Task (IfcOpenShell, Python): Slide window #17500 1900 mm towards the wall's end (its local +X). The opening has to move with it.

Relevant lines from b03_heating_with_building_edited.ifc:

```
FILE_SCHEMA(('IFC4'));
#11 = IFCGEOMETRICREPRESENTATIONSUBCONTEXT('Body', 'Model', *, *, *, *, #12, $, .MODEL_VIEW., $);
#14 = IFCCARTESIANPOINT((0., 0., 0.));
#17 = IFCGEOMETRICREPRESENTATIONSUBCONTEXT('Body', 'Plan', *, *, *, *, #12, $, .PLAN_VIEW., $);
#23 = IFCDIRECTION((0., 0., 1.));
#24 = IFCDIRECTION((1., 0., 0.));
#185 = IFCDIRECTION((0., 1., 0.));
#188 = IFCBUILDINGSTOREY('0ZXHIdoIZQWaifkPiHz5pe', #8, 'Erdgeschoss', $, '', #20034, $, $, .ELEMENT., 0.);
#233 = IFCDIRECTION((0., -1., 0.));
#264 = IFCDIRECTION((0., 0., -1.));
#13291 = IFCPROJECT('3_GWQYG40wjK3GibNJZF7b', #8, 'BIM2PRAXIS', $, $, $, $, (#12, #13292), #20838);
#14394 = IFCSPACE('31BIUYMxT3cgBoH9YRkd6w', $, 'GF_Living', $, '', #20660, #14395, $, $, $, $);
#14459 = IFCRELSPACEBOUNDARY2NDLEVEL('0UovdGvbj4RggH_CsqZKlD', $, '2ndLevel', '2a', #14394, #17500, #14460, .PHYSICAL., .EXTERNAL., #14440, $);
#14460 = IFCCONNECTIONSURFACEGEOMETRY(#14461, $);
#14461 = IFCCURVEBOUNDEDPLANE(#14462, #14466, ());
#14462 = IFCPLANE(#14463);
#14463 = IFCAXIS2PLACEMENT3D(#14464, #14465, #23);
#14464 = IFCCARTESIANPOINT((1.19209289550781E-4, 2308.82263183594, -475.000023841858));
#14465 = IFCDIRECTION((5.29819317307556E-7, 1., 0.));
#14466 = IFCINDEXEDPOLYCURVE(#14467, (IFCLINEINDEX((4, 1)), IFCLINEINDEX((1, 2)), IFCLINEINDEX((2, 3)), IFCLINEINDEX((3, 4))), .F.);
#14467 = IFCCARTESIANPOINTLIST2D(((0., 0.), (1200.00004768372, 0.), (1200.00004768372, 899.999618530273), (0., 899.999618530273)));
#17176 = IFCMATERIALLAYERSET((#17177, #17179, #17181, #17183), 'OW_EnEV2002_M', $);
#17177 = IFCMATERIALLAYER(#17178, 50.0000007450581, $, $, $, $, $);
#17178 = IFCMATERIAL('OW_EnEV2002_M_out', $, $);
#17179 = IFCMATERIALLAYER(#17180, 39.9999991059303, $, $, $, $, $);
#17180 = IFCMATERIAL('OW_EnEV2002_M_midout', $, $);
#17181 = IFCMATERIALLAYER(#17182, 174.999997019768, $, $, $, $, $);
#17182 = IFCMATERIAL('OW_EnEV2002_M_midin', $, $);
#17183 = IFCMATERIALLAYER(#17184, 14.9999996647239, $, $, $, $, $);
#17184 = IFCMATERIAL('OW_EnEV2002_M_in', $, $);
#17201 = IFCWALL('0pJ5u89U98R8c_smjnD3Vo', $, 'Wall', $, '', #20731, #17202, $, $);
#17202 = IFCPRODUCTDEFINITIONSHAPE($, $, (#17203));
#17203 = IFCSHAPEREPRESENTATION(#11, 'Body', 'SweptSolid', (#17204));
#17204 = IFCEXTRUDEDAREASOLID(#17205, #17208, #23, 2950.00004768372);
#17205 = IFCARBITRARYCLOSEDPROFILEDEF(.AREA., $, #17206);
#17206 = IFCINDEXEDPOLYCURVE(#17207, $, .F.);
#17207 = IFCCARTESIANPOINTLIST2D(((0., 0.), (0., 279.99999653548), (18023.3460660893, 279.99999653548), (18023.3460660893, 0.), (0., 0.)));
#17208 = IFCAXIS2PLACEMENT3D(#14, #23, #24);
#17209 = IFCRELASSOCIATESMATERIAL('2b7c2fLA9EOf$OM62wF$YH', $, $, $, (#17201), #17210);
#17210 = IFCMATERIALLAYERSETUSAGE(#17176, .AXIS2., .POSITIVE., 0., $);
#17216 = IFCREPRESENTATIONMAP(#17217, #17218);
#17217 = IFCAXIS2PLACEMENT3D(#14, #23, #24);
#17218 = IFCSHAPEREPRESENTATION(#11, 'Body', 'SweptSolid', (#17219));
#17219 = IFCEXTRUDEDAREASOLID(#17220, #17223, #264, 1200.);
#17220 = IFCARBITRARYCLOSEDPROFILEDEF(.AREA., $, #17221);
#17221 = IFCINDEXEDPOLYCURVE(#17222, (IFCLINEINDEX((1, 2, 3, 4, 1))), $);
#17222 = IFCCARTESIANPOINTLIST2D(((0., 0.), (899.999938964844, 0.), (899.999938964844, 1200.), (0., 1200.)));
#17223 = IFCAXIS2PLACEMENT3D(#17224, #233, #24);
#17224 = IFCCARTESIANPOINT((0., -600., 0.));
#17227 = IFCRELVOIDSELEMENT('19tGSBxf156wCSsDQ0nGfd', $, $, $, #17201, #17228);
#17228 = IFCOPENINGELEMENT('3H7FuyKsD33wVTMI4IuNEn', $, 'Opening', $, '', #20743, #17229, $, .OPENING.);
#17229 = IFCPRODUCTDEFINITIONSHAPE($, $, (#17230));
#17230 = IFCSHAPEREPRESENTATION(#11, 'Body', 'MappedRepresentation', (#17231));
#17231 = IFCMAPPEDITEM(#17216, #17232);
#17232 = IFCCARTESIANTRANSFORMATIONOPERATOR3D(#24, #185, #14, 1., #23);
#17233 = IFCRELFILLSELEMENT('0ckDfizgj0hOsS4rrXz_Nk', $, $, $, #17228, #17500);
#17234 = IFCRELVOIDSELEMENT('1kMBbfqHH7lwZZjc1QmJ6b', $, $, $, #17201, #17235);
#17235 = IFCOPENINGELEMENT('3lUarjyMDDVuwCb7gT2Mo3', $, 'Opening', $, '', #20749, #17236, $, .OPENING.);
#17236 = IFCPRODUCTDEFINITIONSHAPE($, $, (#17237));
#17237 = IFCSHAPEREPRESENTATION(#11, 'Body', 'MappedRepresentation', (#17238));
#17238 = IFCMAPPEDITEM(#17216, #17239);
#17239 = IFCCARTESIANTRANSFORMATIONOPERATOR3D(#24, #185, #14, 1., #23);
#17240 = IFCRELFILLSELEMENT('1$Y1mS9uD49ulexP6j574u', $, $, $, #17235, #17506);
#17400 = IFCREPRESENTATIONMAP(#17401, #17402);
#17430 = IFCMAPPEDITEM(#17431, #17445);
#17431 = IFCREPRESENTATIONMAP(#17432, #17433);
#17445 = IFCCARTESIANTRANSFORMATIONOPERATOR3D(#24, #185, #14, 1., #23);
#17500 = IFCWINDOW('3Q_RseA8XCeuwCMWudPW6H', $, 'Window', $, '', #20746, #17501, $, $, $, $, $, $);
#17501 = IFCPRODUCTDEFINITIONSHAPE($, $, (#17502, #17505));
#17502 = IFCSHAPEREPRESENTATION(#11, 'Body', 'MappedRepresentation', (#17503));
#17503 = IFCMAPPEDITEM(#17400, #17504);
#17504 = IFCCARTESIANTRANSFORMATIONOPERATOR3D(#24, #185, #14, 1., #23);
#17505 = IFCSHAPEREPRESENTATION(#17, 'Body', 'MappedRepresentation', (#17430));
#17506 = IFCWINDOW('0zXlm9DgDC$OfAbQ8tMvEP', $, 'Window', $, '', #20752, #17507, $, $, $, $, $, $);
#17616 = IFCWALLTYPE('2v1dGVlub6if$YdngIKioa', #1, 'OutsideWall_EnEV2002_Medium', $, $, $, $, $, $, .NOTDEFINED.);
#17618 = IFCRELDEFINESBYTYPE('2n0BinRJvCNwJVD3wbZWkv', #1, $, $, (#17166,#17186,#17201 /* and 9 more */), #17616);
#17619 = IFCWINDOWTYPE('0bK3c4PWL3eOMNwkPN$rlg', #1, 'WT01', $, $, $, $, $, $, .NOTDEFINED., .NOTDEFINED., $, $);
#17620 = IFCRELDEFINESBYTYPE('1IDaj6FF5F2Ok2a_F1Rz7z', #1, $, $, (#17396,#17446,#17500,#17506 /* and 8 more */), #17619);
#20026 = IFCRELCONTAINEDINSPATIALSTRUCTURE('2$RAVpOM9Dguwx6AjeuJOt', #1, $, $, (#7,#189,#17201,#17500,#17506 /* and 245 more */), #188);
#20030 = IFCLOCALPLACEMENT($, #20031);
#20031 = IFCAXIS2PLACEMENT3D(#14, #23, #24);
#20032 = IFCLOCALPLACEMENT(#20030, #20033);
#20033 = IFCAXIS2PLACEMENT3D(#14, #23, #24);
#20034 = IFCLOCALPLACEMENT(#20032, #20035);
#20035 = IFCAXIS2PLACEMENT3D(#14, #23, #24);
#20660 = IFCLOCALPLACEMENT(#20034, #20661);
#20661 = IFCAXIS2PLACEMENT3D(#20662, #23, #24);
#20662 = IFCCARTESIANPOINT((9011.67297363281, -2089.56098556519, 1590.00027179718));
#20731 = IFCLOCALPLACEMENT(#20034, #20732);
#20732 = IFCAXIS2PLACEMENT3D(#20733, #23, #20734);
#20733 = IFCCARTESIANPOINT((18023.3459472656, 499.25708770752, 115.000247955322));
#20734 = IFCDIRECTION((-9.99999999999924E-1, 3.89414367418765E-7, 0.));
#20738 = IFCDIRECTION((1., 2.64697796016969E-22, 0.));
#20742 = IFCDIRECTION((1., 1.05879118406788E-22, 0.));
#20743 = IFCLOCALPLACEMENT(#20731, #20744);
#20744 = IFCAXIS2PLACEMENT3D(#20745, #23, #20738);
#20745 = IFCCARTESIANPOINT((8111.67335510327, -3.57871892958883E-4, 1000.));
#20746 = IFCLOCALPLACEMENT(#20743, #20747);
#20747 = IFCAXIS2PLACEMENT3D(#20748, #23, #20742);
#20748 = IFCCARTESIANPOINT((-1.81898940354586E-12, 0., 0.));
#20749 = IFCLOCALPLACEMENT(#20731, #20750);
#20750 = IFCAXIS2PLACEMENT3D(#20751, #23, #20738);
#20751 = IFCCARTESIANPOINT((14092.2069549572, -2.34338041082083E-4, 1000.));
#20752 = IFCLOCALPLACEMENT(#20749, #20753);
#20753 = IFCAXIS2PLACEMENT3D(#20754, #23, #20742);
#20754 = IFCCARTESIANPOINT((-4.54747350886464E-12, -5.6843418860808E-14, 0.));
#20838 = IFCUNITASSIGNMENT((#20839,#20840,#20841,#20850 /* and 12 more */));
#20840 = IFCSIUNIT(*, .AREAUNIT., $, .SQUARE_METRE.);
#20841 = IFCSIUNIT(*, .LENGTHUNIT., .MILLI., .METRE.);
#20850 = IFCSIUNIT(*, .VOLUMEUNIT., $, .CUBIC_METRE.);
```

```python
import numpy as np
import ifcopenshell
import ifcopenshell.api.geometry
import ifcopenshell.util.placement
import ifcopenshell.util.unit

model = ifcopenshell.open("b03_heating_with_building_edited.ifc")
unit_scale = ifcopenshell.util.unit.calculate_unit_scale(model)

window = model.by_id(17500)
opening = window.FillsVoids[0].RelatingOpeningElement
wall = opening.VoidsElements[0].RelatingBuildingElement

wall_matrix = ifcopenshell.util.placement.get_local_placement(wall.ObjectPlacement)
shift = wall_matrix[:3, 0] * 1.9 / unit_scale
before = ifcopenshell.util.placement.get_local_placement(window.ObjectPlacement)[:3, 3].copy()

# The window is placed relative to its opening, so it follows when the opening moves.
matrix = ifcopenshell.util.placement.get_local_placement(opening.ObjectPlacement)
matrix[:3, 3] += shift
ifcopenshell.api.geometry.edit_object_placement(
    model, product=opening, matrix=matrix, is_si=False, should_transform_children=True
)

# Space boundary surfaces are stored in each space's coordinates; move them too.
for rel in window.ProvidesBoundaries:
    if not rel.ConnectionGeometry:
        continue
    surface = rel.ConnectionGeometry.SurfaceOnRelatingElement.BasisSurface
    space_matrix = ifcopenshell.util.placement.get_local_placement(rel.RelatingSpace.ObjectPlacement)
    point = np.array(surface.Position.Location.Coordinates) + space_matrix[:3, :3].T @ shift
    surface.Position = model.createIfcAxis2Placement3D(
        model.createIfcCartesianPoint(point.tolist()), surface.Position.Axis, surface.Position.RefDirection
    )

after = ifcopenshell.util.placement.get_local_placement(window.ObjectPlacement)[:3, 3]
print("window moved by", (after - before).round(3) + 0.0)

model.write("b03_heating_with_building_edited_updated.ifc")
```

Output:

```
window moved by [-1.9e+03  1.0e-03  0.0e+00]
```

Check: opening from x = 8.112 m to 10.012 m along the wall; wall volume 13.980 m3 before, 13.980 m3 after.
